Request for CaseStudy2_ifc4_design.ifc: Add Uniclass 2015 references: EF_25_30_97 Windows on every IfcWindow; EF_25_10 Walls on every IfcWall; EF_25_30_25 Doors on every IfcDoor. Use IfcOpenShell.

First a look at what the model holds.

```python
import ifcopenshell

model = ifcopenshell.open("CaseStudy2_ifc4_design.ifc")
print(model.schema)
print("classifications:", [c.Name for c in model.by_type("IfcClassification")])
for ifc_class in ("IfcDoor", "IfcRoof", "IfcStair", "IfcWall", "IfcWindow"):
    print(ifc_class, len(model.by_type(ifc_class)))
```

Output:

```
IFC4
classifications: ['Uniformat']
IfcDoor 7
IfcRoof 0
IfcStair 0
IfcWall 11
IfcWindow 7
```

```python
import ifcopenshell
import ifcopenshell.api.classification

model = ifcopenshell.open("CaseStudy2_ifc4_design.ifc")

system = ifcopenshell.api.classification.add_classification(model, classification="Uniclass 2015")

codes = {
    "IfcWindow": ("EF_25_30_97", "Windows"),
    "IfcWall": ("EF_25_10", "Walls"),
    "IfcDoor": ("EF_25_30_25", "Doors"),
}
for ifc_class, (code, name) in codes.items():
    products = model.by_type(ifc_class)
    ifcopenshell.api.classification.add_reference(
        model, products=products, classification=system, identification=code, name=name
    )
    print(code, len(products))

model.write("CaseStudy2_ifc4_design-out.ifc")
```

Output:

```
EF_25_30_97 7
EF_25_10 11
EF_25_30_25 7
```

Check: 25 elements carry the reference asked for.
